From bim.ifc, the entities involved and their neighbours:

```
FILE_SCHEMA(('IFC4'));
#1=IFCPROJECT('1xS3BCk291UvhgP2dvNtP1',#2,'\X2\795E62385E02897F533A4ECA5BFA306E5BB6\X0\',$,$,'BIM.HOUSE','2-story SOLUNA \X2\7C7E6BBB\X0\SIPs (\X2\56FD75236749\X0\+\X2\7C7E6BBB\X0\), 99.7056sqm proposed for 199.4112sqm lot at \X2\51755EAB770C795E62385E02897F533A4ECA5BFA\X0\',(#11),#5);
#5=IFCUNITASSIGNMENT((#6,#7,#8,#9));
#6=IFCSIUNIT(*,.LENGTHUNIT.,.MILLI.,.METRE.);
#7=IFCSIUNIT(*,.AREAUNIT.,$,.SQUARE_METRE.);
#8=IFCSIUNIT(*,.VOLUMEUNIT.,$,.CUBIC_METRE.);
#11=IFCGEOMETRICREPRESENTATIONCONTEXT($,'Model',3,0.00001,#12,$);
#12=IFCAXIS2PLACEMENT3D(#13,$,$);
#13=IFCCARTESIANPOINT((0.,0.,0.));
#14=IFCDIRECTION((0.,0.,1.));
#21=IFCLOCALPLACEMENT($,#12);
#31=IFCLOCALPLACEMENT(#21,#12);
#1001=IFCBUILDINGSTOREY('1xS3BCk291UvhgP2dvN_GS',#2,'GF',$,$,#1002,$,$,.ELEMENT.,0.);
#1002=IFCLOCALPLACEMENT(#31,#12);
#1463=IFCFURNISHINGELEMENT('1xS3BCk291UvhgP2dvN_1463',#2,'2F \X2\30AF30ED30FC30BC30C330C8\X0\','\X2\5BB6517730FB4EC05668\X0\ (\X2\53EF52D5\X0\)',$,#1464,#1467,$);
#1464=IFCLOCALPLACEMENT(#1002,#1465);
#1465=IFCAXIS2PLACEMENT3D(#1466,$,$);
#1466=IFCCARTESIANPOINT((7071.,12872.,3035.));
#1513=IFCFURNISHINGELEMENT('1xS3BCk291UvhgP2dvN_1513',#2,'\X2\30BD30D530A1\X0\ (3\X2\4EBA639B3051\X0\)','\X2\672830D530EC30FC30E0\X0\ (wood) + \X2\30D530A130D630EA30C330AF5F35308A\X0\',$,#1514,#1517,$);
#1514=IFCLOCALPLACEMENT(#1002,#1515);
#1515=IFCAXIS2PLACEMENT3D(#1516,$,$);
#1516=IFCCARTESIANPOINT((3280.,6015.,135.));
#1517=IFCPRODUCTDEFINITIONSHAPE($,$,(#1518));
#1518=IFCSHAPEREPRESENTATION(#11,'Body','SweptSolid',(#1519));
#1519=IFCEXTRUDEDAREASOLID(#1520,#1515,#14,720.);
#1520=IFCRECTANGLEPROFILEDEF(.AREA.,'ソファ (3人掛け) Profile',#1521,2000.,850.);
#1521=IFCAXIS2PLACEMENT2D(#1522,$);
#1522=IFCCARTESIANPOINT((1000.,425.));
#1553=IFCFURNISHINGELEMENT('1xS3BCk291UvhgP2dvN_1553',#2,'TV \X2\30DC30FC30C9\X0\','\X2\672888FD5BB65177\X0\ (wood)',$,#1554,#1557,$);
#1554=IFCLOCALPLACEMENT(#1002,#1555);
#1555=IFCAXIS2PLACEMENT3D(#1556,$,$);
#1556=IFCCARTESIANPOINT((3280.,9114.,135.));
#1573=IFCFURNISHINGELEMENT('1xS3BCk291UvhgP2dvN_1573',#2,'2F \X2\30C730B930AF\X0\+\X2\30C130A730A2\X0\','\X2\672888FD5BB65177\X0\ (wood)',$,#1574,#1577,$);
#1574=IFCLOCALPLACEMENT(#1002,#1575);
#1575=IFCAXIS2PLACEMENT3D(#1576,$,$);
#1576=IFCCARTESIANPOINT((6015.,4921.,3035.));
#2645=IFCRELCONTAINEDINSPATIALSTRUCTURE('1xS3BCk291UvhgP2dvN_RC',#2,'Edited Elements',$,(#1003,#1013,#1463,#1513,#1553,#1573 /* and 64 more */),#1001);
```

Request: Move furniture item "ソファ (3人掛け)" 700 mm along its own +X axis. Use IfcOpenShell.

```python
import ifcopenshell
import ifcopenshell.api.geometry
import ifcopenshell.util.placement
import ifcopenshell.util.unit

model = ifcopenshell.open("bim.ifc")
unit_scale = ifcopenshell.util.unit.calculate_unit_scale(model)

item = model.by_guid("1xS3BCk291UvhgP2dvN_1513")
matrix = ifcopenshell.util.placement.get_local_placement(item.ObjectPlacement)
matrix[:3, 3] += matrix[:3, 0] * 0.7 / unit_scale
ifcopenshell.api.geometry.edit_object_placement(model, product=item, matrix=matrix, is_si=False)

print(ifcopenshell.util.placement.get_local_placement(item.ObjectPlacement).round(3) + 0.0)

model.write("bim-out.ifc")
```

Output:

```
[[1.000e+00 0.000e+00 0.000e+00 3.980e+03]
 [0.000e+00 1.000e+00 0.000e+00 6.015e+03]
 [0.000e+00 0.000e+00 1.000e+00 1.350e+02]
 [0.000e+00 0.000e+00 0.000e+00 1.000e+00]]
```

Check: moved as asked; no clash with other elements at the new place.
